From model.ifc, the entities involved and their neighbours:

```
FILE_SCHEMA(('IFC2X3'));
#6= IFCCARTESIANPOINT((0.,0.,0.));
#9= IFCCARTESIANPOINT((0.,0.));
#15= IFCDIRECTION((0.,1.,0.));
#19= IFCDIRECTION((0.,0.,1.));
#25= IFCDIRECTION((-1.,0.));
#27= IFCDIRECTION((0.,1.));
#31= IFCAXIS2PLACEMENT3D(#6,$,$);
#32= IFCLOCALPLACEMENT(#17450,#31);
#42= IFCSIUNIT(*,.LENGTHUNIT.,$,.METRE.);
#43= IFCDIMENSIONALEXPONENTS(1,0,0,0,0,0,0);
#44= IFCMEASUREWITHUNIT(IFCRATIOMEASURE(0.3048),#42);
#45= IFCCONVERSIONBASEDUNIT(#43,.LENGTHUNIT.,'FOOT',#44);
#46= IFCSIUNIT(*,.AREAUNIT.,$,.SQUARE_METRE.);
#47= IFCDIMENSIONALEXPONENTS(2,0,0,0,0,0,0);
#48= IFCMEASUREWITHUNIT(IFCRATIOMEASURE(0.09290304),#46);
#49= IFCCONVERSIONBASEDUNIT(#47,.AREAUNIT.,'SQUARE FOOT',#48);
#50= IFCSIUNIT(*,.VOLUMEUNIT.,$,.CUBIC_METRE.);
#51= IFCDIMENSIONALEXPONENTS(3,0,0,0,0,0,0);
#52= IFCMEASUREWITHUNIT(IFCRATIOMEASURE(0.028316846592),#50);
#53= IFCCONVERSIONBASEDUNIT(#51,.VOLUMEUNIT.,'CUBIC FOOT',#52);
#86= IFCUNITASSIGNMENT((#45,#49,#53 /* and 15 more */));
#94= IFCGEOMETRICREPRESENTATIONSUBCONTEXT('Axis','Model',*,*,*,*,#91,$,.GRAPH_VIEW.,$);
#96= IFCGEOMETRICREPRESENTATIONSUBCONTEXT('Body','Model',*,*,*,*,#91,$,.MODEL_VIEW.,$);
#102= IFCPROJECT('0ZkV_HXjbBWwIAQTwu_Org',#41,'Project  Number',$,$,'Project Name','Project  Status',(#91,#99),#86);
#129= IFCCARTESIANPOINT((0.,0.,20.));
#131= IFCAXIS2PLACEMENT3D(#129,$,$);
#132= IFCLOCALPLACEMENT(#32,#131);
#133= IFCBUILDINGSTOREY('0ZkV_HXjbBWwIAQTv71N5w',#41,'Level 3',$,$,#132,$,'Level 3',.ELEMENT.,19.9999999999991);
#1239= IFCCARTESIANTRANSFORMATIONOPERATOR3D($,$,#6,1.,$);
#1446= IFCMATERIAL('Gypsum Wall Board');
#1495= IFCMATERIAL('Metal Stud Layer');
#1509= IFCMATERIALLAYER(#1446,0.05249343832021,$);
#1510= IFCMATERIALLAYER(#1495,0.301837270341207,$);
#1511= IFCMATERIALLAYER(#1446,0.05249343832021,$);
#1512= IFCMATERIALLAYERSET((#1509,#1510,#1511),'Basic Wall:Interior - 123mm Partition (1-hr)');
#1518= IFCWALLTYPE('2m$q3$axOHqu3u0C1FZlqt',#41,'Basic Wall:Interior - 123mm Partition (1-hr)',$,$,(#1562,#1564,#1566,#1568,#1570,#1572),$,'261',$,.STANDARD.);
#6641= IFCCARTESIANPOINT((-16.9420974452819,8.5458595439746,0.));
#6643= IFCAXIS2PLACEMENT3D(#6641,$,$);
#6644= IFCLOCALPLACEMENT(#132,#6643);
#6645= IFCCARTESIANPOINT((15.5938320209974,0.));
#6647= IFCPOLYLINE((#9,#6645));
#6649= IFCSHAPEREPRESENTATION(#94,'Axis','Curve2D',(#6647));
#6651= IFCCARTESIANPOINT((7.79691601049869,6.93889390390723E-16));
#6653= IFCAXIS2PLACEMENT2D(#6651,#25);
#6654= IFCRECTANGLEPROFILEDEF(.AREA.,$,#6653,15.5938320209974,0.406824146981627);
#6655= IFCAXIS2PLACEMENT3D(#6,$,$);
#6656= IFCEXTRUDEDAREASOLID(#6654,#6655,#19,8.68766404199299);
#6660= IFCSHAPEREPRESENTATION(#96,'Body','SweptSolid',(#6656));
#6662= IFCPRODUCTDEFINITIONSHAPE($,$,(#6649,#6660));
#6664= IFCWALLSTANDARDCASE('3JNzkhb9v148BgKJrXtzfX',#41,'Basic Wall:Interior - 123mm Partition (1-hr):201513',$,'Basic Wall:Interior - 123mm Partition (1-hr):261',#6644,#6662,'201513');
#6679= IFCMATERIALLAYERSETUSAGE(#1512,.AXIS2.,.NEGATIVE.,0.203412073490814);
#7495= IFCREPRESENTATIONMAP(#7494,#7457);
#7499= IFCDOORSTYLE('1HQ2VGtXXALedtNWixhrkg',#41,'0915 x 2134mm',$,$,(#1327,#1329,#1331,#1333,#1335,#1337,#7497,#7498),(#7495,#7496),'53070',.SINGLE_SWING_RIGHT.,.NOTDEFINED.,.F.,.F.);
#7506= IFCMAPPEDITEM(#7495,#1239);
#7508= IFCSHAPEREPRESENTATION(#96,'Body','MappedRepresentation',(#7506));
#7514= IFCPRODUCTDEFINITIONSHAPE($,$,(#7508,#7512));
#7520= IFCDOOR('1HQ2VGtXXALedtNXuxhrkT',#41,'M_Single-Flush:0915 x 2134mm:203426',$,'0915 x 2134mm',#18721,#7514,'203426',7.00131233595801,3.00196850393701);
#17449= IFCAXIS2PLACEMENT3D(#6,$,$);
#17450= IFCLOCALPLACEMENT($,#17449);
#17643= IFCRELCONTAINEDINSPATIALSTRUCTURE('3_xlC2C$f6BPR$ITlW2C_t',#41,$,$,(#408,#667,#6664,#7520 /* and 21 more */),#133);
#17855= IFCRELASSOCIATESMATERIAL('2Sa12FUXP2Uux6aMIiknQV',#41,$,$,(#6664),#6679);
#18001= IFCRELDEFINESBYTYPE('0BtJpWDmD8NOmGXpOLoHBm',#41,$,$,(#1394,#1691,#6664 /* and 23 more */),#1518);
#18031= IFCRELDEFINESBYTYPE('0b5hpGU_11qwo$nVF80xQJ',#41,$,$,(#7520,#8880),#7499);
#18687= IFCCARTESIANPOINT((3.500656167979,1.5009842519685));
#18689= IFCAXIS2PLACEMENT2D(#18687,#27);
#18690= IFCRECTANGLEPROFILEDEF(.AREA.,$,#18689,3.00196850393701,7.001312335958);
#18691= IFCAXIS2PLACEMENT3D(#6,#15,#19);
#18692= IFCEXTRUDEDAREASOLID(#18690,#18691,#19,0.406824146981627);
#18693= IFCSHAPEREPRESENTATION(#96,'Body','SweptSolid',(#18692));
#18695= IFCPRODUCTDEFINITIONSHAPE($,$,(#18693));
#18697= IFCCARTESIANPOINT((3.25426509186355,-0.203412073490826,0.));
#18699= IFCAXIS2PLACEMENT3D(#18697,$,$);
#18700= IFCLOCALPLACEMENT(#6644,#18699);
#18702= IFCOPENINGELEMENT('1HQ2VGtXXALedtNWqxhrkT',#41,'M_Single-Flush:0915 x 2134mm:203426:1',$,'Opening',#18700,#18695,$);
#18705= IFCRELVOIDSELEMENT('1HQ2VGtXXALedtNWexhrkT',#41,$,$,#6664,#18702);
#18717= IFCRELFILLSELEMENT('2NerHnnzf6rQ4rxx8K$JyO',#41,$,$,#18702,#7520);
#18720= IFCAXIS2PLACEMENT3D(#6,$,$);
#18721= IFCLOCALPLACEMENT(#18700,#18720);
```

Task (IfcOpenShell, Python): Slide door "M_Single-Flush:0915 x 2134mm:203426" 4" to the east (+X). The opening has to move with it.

```python
import ifcopenshell
import ifcopenshell.api.geometry
import ifcopenshell.util.placement
import ifcopenshell.util.unit

model = ifcopenshell.open("model.ifc")
unit_scale = ifcopenshell.util.unit.calculate_unit_scale(model)

door = model.by_guid("1HQ2VGtXXALedtNXuxhrkT")
opening = door.FillsVoids[0].RelatingOpeningElement
wall = opening.VoidsElements[0].RelatingBuildingElement

wall_matrix = ifcopenshell.util.placement.get_local_placement(wall.ObjectPlacement)
shift = wall_matrix[:3, 0] * 4 * 0.0254 / unit_scale
before = ifcopenshell.util.placement.get_local_placement(door.ObjectPlacement)[:3, 3].copy()

# The door is placed relative to its opening, so it follows when the opening moves.
matrix = ifcopenshell.util.placement.get_local_placement(opening.ObjectPlacement)
matrix[:3, 3] += shift
ifcopenshell.api.geometry.edit_object_placement(
    model, product=opening, matrix=matrix, is_si=False, should_transform_children=True
)

after = ifcopenshell.util.placement.get_local_placement(door.ObjectPlacement)[:3, 3]
print("door moved by", (after - before).round(3) + 0.0)

model.write("model_rev.ifc")
```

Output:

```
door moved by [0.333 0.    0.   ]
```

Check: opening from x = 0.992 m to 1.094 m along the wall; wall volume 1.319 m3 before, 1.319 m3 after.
